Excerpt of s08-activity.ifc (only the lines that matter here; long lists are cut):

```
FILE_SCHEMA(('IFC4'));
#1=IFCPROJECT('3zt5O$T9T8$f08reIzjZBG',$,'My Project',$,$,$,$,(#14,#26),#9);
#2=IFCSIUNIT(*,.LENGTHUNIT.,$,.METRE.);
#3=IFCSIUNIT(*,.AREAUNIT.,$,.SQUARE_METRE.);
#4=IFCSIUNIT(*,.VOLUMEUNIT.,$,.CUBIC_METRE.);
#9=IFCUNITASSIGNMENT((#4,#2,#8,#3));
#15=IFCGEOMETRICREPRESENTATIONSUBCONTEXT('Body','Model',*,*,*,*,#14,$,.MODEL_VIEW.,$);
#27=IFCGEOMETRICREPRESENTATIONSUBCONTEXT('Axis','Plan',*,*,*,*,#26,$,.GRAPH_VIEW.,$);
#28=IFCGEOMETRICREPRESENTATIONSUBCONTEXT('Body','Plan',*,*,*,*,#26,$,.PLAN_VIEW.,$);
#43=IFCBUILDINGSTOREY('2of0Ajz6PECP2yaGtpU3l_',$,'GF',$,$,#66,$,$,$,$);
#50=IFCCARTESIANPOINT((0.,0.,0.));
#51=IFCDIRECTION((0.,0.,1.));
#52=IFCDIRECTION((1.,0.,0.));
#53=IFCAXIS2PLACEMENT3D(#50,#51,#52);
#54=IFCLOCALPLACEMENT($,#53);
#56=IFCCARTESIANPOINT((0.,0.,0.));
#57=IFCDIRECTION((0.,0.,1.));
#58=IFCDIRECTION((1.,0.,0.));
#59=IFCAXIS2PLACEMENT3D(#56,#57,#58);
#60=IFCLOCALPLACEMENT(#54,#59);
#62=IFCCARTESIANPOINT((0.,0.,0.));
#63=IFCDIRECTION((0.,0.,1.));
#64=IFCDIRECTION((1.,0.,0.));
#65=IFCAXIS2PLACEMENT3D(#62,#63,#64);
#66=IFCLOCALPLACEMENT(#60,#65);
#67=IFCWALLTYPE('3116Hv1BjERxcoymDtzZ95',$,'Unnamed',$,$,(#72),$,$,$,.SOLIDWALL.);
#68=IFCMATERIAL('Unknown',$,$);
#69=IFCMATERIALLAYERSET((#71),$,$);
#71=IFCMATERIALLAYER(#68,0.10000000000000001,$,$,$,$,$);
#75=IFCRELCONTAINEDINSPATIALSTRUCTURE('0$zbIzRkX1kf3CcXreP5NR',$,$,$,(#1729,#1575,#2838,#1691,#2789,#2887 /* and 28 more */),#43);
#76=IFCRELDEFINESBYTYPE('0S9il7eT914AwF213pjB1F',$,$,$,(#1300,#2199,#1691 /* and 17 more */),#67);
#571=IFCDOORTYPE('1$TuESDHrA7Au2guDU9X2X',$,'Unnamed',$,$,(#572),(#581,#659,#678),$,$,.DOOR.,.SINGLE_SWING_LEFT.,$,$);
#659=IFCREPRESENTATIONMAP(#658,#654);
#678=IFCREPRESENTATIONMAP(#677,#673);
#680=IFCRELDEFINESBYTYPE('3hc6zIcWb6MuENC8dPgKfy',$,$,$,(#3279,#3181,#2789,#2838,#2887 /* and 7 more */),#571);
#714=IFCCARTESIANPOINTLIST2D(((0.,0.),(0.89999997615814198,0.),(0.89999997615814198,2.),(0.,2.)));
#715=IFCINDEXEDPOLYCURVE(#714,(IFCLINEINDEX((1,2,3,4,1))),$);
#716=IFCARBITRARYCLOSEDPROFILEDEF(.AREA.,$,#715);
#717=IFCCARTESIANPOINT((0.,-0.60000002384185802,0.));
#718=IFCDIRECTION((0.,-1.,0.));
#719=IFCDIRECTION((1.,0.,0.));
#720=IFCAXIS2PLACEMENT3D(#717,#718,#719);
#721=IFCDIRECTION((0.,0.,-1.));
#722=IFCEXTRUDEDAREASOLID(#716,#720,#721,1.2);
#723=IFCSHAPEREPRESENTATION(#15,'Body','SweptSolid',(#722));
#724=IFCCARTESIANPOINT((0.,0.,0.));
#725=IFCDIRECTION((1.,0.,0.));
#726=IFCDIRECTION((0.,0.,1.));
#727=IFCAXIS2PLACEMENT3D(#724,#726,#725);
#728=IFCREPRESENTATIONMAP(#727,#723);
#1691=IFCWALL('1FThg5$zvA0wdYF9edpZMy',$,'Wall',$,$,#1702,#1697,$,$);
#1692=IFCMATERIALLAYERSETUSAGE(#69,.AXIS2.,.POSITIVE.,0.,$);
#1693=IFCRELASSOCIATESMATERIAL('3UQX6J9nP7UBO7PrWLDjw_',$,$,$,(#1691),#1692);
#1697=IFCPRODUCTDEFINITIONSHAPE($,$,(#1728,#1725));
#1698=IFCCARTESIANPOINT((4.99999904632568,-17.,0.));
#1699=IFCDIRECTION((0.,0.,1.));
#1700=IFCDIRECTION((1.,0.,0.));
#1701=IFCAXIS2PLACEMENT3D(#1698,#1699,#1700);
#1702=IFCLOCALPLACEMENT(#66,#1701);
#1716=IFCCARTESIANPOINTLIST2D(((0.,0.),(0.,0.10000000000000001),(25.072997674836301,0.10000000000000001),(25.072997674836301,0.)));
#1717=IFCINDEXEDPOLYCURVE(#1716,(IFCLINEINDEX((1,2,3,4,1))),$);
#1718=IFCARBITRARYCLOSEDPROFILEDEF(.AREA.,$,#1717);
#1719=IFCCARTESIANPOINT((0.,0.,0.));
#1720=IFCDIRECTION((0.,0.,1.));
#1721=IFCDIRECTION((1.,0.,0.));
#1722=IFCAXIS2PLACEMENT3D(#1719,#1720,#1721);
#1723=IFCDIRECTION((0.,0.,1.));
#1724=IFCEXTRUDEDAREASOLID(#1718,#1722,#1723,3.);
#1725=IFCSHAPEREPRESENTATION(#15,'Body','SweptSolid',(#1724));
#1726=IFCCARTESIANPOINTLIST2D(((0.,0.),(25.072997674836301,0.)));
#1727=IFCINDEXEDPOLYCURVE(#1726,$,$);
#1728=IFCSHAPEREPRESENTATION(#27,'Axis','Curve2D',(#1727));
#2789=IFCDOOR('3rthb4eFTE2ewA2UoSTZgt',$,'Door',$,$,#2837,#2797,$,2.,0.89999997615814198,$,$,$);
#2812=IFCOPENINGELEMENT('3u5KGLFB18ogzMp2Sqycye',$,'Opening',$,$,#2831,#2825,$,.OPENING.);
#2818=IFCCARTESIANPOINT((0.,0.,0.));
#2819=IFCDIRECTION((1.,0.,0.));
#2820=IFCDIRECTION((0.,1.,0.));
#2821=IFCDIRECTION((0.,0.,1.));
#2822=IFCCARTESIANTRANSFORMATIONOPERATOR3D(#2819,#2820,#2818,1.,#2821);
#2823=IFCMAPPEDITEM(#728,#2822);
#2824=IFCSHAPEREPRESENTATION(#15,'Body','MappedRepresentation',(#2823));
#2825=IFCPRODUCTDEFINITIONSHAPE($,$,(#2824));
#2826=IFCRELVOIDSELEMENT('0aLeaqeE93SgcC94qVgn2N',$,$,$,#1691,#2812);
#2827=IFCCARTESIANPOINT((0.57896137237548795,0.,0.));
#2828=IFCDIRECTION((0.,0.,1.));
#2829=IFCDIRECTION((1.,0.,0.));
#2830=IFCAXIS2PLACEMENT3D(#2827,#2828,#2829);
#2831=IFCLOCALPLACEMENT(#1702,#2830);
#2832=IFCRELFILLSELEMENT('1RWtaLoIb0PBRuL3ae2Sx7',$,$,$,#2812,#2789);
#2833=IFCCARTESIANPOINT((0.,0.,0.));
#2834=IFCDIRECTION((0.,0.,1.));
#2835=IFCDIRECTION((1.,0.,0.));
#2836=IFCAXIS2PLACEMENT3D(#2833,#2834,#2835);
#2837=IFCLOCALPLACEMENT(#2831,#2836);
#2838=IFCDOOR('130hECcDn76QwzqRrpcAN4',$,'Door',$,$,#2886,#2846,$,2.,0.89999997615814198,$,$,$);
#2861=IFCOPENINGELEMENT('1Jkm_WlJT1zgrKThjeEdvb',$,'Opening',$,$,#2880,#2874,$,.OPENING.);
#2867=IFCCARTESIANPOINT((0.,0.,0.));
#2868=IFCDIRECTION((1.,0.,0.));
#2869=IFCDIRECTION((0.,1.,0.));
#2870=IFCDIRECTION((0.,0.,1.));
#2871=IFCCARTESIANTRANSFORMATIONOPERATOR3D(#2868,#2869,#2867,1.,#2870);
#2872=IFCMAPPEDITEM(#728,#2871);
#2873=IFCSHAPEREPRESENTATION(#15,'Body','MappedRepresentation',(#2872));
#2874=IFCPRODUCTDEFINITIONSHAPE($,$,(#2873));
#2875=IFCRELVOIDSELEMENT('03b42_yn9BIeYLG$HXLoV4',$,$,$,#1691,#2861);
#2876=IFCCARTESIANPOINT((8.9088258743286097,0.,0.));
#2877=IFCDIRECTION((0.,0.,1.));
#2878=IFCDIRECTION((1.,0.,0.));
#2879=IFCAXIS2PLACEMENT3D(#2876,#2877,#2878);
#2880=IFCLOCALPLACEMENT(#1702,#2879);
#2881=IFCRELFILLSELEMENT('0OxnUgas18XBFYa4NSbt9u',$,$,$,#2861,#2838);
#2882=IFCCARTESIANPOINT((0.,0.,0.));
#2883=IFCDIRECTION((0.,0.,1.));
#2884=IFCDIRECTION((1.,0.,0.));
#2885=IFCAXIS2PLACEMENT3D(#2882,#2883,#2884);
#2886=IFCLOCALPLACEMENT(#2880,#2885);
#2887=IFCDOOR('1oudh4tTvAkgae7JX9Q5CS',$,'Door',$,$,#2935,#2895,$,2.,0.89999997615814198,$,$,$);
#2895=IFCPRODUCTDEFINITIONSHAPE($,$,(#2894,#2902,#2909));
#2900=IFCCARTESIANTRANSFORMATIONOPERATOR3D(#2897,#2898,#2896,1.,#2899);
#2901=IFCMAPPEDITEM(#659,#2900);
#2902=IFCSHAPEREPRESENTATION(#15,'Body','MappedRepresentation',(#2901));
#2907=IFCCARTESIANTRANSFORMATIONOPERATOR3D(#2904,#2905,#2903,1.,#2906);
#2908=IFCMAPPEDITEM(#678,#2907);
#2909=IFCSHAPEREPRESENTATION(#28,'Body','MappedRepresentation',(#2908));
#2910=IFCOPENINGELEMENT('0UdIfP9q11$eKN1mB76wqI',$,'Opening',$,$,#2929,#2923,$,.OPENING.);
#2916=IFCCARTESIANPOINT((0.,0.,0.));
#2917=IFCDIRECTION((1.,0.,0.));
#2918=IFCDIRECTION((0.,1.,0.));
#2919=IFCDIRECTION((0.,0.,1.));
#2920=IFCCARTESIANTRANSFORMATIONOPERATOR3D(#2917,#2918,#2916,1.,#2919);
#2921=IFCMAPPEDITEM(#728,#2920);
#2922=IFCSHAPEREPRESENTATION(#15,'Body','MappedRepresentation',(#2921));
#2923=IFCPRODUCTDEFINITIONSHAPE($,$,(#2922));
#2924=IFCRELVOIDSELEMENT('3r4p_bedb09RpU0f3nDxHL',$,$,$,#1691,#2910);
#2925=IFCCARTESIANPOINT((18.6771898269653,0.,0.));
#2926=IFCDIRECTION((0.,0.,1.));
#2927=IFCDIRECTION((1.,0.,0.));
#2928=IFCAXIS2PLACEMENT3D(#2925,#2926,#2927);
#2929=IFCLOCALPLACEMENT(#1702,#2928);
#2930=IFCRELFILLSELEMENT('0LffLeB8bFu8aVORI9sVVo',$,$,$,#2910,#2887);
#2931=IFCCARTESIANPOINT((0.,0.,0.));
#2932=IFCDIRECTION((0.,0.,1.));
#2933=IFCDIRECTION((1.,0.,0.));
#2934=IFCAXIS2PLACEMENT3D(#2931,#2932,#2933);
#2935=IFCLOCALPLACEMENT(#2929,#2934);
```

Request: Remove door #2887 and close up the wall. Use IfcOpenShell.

```python
import ifcopenshell
import ifcopenshell.api.feature
import ifcopenshell.api.root
import ifcopenshell.geom
import ifcopenshell.util.shape

model = ifcopenshell.open("s08-activity.ifc")
settings = ifcopenshell.geom.settings()


def volume(element):
    """Net volume in cubic metres, openings subtracted."""
    shape = ifcopenshell.geom.create_shape(settings, element)
    return ifcopenshell.util.shape.get_volume(shape.geometry)


door = model.by_guid("1oudh4tTvAkgae7JX9Q5CS")
opening = door.FillsVoids[0].RelatingOpeningElement
wall = opening.VoidsElements[0].RelatingBuildingElement
before = volume(wall)

ifcopenshell.api.root.remove_product(model, product=door)
ifcopenshell.api.feature.remove_feature(model, feature=opening)

after = volume(wall)

print(f"wall volume {before:.3f} -> {after:.3f} m3")

model.write("s08-activity_updated.ifc")
```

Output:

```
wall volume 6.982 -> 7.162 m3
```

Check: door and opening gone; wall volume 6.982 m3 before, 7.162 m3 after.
